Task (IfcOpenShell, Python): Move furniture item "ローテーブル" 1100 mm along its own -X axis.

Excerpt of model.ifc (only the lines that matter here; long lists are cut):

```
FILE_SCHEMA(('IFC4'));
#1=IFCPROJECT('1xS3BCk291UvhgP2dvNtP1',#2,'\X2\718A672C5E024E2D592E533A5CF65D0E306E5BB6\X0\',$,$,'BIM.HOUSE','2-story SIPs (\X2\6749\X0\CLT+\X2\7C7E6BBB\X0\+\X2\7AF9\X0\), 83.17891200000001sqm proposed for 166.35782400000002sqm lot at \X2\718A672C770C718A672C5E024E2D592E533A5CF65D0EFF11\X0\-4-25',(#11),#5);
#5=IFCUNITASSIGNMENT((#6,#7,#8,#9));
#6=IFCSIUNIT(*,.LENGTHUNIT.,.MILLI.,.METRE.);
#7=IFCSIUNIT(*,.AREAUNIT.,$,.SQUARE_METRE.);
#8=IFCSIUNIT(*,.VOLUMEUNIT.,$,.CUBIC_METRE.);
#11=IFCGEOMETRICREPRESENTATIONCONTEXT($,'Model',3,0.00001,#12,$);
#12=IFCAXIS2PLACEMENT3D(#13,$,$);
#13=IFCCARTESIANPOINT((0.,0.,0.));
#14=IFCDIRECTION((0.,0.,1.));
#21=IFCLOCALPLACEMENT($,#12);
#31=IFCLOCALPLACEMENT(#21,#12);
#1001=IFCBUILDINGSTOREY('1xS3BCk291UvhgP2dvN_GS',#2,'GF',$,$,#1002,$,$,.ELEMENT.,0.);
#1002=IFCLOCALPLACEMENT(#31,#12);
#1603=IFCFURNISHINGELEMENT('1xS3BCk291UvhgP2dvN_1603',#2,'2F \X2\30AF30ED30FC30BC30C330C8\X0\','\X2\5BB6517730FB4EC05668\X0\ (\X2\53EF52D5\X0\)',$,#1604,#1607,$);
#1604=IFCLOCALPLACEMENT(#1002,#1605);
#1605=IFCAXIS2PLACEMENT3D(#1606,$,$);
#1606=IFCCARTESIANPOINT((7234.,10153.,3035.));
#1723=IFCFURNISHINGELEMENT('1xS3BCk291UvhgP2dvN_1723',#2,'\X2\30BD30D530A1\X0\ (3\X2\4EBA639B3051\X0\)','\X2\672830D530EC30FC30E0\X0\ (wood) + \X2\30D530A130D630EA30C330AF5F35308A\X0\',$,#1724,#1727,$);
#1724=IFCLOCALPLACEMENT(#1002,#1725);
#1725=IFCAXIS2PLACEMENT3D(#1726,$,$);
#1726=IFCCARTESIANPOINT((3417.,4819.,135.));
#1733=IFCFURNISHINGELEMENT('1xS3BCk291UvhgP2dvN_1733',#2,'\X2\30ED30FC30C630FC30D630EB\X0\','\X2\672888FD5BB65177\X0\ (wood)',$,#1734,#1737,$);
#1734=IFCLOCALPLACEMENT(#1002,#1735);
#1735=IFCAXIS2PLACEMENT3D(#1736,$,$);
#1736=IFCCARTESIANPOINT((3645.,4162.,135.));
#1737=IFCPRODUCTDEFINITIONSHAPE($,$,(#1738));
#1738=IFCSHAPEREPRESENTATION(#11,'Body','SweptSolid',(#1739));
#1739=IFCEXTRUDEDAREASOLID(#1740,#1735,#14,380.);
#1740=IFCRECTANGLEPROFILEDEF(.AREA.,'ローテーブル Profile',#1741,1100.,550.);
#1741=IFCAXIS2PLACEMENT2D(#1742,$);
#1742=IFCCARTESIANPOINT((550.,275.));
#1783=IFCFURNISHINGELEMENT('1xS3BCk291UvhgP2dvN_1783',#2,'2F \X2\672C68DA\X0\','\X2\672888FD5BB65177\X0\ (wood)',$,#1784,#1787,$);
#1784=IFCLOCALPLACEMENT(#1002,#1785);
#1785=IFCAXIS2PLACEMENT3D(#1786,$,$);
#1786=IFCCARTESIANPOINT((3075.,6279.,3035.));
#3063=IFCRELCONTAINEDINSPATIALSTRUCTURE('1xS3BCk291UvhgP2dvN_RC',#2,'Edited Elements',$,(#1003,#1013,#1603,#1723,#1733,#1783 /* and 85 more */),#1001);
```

```python
import ifcopenshell
import ifcopenshell.api.geometry
import ifcopenshell.util.placement

model = ifcopenshell.open("model.ifc")

item = model.by_id(1733)
matrix = ifcopenshell.util.placement.get_local_placement(item.ObjectPlacement)
matrix[:3, 3] -= matrix[:3, 0] * 1100.0
ifcopenshell.api.geometry.edit_object_placement(model, product=item, matrix=matrix, is_si=False)

print(ifcopenshell.util.placement.get_local_placement(item.ObjectPlacement).round(3) + 0.0)

model.write("model_updated.ifc")
```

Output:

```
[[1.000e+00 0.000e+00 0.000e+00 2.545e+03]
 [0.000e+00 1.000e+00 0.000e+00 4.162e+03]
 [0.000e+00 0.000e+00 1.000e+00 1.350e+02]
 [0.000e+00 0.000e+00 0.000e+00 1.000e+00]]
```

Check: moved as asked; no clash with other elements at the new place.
